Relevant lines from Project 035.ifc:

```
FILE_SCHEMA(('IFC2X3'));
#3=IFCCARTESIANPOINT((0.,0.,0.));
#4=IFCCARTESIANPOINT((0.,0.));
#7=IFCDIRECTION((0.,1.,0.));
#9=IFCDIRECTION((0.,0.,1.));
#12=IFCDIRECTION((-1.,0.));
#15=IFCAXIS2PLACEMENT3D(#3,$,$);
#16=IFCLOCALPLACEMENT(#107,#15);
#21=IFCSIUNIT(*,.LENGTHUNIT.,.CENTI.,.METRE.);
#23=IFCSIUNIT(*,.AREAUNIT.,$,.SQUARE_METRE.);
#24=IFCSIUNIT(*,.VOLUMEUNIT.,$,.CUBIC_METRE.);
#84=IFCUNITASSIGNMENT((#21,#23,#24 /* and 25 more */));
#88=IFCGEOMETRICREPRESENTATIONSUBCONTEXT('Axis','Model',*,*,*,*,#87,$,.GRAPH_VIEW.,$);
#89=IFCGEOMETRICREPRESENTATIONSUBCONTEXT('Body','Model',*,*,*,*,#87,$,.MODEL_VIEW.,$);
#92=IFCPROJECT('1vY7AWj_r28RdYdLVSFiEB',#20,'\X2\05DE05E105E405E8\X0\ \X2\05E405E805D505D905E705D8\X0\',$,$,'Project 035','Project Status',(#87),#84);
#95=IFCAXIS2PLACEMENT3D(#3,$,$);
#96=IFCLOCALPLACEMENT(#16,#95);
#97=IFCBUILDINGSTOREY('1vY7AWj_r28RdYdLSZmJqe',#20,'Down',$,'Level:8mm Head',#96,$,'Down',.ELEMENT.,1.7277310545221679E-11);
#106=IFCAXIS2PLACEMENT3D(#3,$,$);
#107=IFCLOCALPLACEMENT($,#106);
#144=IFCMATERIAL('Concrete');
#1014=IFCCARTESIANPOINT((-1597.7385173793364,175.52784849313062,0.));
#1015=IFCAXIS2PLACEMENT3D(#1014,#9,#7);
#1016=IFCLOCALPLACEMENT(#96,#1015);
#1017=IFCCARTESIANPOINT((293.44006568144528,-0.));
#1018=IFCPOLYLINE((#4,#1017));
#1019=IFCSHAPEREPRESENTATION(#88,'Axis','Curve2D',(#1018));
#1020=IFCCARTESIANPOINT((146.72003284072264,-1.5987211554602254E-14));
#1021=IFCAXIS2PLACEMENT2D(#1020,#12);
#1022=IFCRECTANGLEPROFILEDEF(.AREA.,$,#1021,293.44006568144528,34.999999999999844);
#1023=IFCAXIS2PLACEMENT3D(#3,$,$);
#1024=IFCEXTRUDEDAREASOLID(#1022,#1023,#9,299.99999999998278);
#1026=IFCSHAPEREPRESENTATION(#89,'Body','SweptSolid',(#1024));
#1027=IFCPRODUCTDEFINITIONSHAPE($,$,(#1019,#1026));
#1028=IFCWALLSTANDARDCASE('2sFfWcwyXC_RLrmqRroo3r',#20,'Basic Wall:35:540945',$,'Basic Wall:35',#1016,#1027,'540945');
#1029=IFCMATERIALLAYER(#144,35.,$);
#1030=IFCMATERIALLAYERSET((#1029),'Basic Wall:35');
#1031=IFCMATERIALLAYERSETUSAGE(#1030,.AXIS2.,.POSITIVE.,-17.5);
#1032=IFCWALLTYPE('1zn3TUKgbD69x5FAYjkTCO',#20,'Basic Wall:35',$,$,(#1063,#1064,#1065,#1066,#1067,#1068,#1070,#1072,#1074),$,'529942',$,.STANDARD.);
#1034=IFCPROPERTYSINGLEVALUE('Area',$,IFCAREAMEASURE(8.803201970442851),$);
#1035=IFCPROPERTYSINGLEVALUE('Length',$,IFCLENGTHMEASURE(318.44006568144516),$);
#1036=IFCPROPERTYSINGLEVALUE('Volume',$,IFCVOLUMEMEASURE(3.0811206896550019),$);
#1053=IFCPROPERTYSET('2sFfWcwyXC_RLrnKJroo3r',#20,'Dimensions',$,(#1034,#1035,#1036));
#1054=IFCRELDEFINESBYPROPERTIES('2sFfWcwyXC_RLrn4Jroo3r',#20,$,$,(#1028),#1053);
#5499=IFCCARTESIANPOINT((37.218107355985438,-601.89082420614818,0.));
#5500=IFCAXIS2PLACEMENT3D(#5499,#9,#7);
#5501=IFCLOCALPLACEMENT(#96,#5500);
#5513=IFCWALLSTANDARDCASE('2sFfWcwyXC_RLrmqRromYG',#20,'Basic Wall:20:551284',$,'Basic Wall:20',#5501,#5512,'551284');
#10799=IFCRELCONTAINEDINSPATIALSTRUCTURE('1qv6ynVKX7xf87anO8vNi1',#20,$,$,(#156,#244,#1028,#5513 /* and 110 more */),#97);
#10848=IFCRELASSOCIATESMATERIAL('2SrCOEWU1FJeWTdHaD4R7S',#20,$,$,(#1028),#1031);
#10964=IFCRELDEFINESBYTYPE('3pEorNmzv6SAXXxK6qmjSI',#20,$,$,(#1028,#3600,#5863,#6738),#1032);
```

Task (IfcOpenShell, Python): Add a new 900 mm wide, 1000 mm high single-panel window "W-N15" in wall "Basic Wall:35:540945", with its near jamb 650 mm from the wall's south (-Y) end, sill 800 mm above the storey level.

```python
import numpy as np
import ifcopenshell
import ifcopenshell.api.feature
import ifcopenshell.api.geometry
import ifcopenshell.api.pset
import ifcopenshell.api.root
import ifcopenshell.api.spatial
import ifcopenshell.api.type
import ifcopenshell.geom
import ifcopenshell.util.element
import ifcopenshell.util.placement
import ifcopenshell.util.representation
import ifcopenshell.util.shape
import ifcopenshell.util.unit

model = ifcopenshell.open("Project 035.ifc")
unit_scale = ifcopenshell.util.unit.calculate_unit_scale(model)
area_scale = ifcopenshell.util.unit.calculate_unit_scale(model, "AREAUNIT")
volume_scale = ifcopenshell.util.unit.calculate_unit_scale(model, "VOLUMEUNIT")
settings = ifcopenshell.geom.settings()


def volume(element):
    """Net volume in cubic metres, openings subtracted."""
    shape = ifcopenshell.geom.create_shape(settings, element)
    return ifcopenshell.util.shape.get_volume(shape.geometry)


wall = model.by_id(1028)
storey = ifcopenshell.util.element.get_container(wall, ifc_class="IfcBuildingStorey")
context = ifcopenshell.util.representation.get_context(model, "Model", "Body", "MODEL_VIEW")
before = volume(wall)

width, height, from_end, sill = 0.9, 1, 0.65, 0.8  # metres

# The wall runs along its own X axis, and the end named is its -X end.
wall_shape = ifcopenshell.geom.create_shape(settings, wall)
x, y, z = ifcopenshell.util.shape.get_vertices(wall_shape.geometry).T
start = x.min() + from_end
face, thickness = float(y.min()), float(y.max() - y.min())
wall_matrix = ifcopenshell.util.placement.get_local_placement(wall.ObjectPlacement)
level = ifcopenshell.util.placement.get_local_placement(storey.ObjectPlacement)[2, 3]


def in_wall(x, y):
    """Placement at x, y metres in the wall's axes, at sill height."""
    matrix = wall_matrix.copy()
    matrix[:, 3] = wall_matrix @ np.array([x / unit_scale, y / unit_scale, 0.0, 1.0])
    matrix[2, 3] = level + sill / unit_scale
    return matrix


# Opening: a box that overshoots both wall faces by 50 mm.
opening = ifcopenshell.api.root.create_entity(model, ifc_class="IfcOpeningElement")
box = ifcopenshell.api.geometry.add_wall_representation(
    model, context=context, length=width, height=height, thickness=thickness + 0.1
)
ifcopenshell.api.geometry.assign_representation(model, product=opening, representation=box)
ifcopenshell.api.geometry.edit_object_placement(model, product=opening, matrix=in_wall(start, face - 0.05), is_si=False)
ifcopenshell.api.feature.add_feature(model, feature=opening, element=wall)

window = ifcopenshell.api.root.create_entity(model, ifc_class="IfcWindow", name="W-N15")
window.OverallWidth, window.OverallHeight = width / unit_scale, height / unit_scale
body = ifcopenshell.api.geometry.add_window_representation(
    model,
    context=context,
    overall_width=window.OverallWidth,
    overall_height=window.OverallHeight,
    partition_type="SINGLE_PANEL",
)
ifcopenshell.api.geometry.assign_representation(model, product=window, representation=body)
ifcopenshell.api.spatial.assign_container(model, products=[window], relating_structure=storey)
fills = ifcopenshell.api.feature.add_filling(model, opening=opening, element=window)
fills.OwnerHistory = window.OwnerHistory  # required in IFC2X3

# IFC2X3 keeps the operation on the window style.
style = ifcopenshell.api.root.create_entity(model, ifc_class="IfcWindowStyle", name="W-N15")
style.OperationType, style.ConstructionType = "SINGLE_PANEL", "NOTDEFINED"
style.ParameterTakesPrecedence = style.Sizeable = False
ifcopenshell.api.type.assign_type(model, related_objects=[window], relating_type=style)

# Centre the window in the wall's thickness.
ifcopenshell.api.geometry.edit_object_placement(model, product=window, matrix=in_wall(start, face), is_si=False)
window_shape = ifcopenshell.geom.create_shape(settings, window)
depth = ifcopenshell.util.shape.get_vertices(window_shape.geometry)[:, 1]
offset = face + thickness / 2 - (depth.min() + depth.max()) / 2
ifcopenshell.api.geometry.edit_object_placement(model, product=window, matrix=in_wall(start, offset), is_si=False)

after = volume(wall)

# Update the wall's stored quantities.
pset = model.by_id(ifcopenshell.util.element.get_pset(wall, "Dimensions", should_inherit=False)["id"])
ifcopenshell.api.pset.edit_pset(model, pset=pset, properties={
    "Area": model.create_entity("IfcAreaMeasure", after / thickness / area_scale),
    "Volume": model.create_entity("IfcVolumeMeasure", after / volume_scale),
})

print(f"wall volume {before:.3f} -> {after:.3f} m3")

model.write("Project 035_updated.ifc")
```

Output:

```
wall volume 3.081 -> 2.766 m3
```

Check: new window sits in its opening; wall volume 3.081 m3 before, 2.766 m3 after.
